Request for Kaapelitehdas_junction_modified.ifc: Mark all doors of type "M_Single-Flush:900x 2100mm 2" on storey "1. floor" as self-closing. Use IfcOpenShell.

First a look at what the model holds.

```python
import ifcopenshell
import ifcopenshell.util.element

model = ifcopenshell.open("Kaapelitehdas_junction_modified.ifc")
print(model.schema)
storey = next(s for s in model.by_type("IfcBuildingStorey") if s.Name == "1. floor")
doors = [e for e in ifcopenshell.util.element.get_decomposition(storey) if e.is_a("IfcDoor")]
seen = {}
for e in doors:
    element_type = ifcopenshell.util.element.get_type(e)
    key = (element_type.Name if element_type != e and element_type else None, ifcopenshell.util.element.get_pset(e, "Pset_DoorCommon", "SelfClosing"))
    seen[key] = seen.get(key, 0) + 1
for (name, value), count in sorted(seen.items(), key=str):
    print(count, "x", name, "|", value)
```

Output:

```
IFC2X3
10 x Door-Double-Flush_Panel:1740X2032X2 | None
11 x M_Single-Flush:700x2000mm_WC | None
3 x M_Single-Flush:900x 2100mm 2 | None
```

```python
import ifcopenshell
import ifcopenshell.api.pset
import ifcopenshell.util.element

model = ifcopenshell.open("Kaapelitehdas_junction_modified.ifc")

storey = next(s for s in model.by_type("IfcBuildingStorey") if s.Name == "1. floor")
doors = [e for e in ifcopenshell.util.element.get_decomposition(storey) if e.is_a("IfcDoor")]

count = 0
for e in doors:
    element_type = ifcopenshell.util.element.get_type(e)
    if element_type in (None, e) or element_type.Name != "M_Single-Flush:900x 2100mm 2":
        continue
    # add_pset returns the element's existing set when there is one.
    pset = ifcopenshell.api.pset.add_pset(model, product=e, name="Pset_DoorCommon")
    ifcopenshell.api.pset.edit_pset(model, pset=pset, properties={"SelfClosing": True})
    count += 1

print(count, "doors updated")

model.write("Kaapelitehdas_junction_modified-out.ifc")
```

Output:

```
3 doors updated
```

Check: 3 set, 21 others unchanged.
